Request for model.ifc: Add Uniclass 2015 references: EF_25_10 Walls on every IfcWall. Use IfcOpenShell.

First a look at what the model holds.

```python
import ifcopenshell

model = ifcopenshell.open("model.ifc")
print(model.schema)
print("classifications:", [c.Name for c in model.by_type("IfcClassification")])
for ifc_class in ("IfcDoor", "IfcRoof", "IfcStair", "IfcWall", "IfcWindow"):
    print(ifc_class, len(model.by_type(ifc_class)))
```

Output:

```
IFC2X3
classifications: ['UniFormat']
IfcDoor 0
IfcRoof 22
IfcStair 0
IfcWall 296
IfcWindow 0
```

```python
import ifcopenshell
import ifcopenshell.api.classification

model = ifcopenshell.open("model.ifc")

# IFC2X3 requires Source and Edition and has no link from the project to the system.
system = model.create_entity("IfcClassification", Source="NBS", Edition="2015", Name="Uniclass 2015")

codes = {
    "IfcWall": ("EF_25_10", "Walls"),
}
for ifc_class, (code, name) in codes.items():
    products = model.by_type(ifc_class)
    ifcopenshell.api.classification.add_reference(
        model, products=products, classification=system, identification=code, name=name
    )
    print(code, len(products))

model.write("model_v2.ifc")
```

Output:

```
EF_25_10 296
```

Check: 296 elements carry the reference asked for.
